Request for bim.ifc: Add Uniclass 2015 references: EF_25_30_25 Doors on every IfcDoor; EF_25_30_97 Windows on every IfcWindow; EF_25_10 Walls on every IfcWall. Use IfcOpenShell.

First a look at what the model holds.

```python
import ifcopenshell

model = ifcopenshell.open("bim.ifc")
print(model.schema)
print("classifications:", [c.Name for c in model.by_type("IfcClassification")])
for ifc_class in ("IfcDoor", "IfcRoof", "IfcStair", "IfcWall", "IfcWindow"):
    print(ifc_class, len(model.by_type(ifc_class)))
```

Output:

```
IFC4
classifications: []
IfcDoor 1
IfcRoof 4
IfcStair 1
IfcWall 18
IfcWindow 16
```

```python
import ifcopenshell
import ifcopenshell.api.classification

model = ifcopenshell.open("bim.ifc")

system = ifcopenshell.api.classification.add_classification(model, classification="Uniclass 2015")

codes = {
    "IfcDoor": ("EF_25_30_25", "Doors"),
    "IfcWindow": ("EF_25_30_97", "Windows"),
    "IfcWall": ("EF_25_10", "Walls"),
}
for ifc_class, (code, name) in codes.items():
    products = model.by_type(ifc_class)
    ifcopenshell.api.classification.add_reference(
        model, products=products, classification=system, identification=code, name=name
    )
    print(code, len(products))

model.write("bim_rev.ifc")
```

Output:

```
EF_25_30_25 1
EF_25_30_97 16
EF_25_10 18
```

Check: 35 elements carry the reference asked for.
